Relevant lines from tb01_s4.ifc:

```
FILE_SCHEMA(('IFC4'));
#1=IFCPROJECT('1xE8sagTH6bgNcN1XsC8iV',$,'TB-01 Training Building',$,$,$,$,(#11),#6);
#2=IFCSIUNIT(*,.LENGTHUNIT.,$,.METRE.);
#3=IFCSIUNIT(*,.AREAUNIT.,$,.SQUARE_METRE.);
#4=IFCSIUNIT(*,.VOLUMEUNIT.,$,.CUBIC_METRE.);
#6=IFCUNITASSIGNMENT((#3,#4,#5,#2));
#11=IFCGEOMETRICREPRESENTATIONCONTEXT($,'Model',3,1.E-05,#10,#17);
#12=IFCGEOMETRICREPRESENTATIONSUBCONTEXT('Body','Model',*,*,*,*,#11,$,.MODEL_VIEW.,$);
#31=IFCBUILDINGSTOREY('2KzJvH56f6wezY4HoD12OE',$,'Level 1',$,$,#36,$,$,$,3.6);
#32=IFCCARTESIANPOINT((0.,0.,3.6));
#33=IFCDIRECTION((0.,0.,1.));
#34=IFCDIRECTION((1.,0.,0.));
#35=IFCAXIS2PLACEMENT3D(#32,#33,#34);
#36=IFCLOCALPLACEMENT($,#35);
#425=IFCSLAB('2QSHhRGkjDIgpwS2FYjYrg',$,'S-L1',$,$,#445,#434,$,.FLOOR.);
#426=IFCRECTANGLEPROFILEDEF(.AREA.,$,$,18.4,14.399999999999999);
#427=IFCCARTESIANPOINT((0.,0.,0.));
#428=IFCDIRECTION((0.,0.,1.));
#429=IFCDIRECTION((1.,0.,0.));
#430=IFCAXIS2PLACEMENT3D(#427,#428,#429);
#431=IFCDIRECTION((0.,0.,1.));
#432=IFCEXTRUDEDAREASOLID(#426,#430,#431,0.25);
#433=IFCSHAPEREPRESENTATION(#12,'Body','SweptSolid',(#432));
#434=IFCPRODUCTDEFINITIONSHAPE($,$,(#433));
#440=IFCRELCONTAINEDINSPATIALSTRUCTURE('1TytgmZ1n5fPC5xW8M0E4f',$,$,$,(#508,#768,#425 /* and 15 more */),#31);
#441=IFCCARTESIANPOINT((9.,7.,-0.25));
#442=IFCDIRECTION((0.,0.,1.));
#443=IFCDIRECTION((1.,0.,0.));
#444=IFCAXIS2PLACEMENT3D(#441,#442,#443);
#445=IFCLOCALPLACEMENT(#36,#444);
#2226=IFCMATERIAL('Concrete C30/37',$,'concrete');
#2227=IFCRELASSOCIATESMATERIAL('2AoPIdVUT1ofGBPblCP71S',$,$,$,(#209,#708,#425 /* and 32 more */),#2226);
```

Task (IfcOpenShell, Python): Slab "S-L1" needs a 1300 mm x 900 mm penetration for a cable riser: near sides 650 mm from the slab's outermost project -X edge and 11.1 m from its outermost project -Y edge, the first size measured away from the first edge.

```python
import numpy as np
import ifcopenshell
import ifcopenshell.api.feature
import ifcopenshell.api.geometry
import ifcopenshell.api.root
import ifcopenshell.geom
import ifcopenshell.util.placement
import ifcopenshell.util.representation
import ifcopenshell.util.shape
import ifcopenshell.util.unit

model = ifcopenshell.open("tb01_s4.ifc")
unit_scale = ifcopenshell.util.unit.calculate_unit_scale(model)
settings = ifcopenshell.geom.settings()


def volume(element):
    """Net volume in cubic metres, openings subtracted."""
    shape = ifcopenshell.geom.create_shape(settings, element)
    return ifcopenshell.util.shape.get_volume(shape.geometry)


slab = model.by_guid("2QSHhRGkjDIgpwS2FYjYrg")
before = volume(slab)

# Extent in the slab's own axes, in metres. The edges named are its -X and -Y sides.
slab_shape = ifcopenshell.geom.create_shape(settings, slab)
vertices = ifcopenshell.util.shape.get_vertices(slab_shape.geometry)
x_min, y_min, bottom = vertices.min(axis=0)
top = vertices[:, 2].max()

opening = ifcopenshell.api.root.create_entity(model, ifc_class="IfcOpeningElement", name="Cable riser opening", predefined_type="OPENING")
context = ifcopenshell.util.representation.get_context(model, "Model", "Body", "MODEL_VIEW")
width, depth = 1.3, 0.9
outline = [(0.0, 0.0), (width, 0.0), (width, depth), (0.0, depth), (0.0, 0.0)]
# Overshoot both faces by 50 mm so the cut is clean.
shape = ifcopenshell.api.geometry.add_slab_representation(
    model, context=context, depth=top - bottom + 0.1, polyline=outline
)
ifcopenshell.api.geometry.assign_representation(model, product=opening, representation=shape)

matrix = ifcopenshell.util.placement.get_local_placement(slab.ObjectPlacement)
matrix[:, 3] = matrix @ np.append(np.array([x_min + 0.65, y_min + 11.1, bottom - 0.05]) / unit_scale, 1.0)
ifcopenshell.api.geometry.edit_object_placement(model, product=opening, matrix=matrix, is_si=False)
ifcopenshell.api.feature.add_feature(model, feature=opening, element=slab)

after = volume(slab)

print(f"slab volume {before:.3f} -> {after:.3f} m3")

model.write("tb01_s4-out.ifc")
```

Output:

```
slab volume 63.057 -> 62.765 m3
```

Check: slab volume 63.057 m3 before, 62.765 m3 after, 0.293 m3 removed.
